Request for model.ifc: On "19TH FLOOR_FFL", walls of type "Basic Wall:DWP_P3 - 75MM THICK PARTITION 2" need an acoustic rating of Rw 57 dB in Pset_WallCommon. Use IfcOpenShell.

First a look at what the model holds.

```python
import ifcopenshell
import ifcopenshell.util.element

model = ifcopenshell.open("model.ifc")
print(model.schema)
storey = next(s for s in model.by_type("IfcBuildingStorey") if s.Name == "19TH FLOOR_FFL")
walls = [e for e in ifcopenshell.util.element.get_decomposition(storey) if e.is_a("IfcWall")]
seen = {}
for e in walls:
    element_type = ifcopenshell.util.element.get_type(e)
    key = (element_type.Name if element_type != e and element_type else None, ifcopenshell.util.element.get_pset(e, "Pset_WallCommon", "AcousticRating"))
    seen[key] = seen.get(key, 0) + 1
for (name, value), count in sorted(seen.items(), key=str):
    print(count, "x", name, "|", value)
```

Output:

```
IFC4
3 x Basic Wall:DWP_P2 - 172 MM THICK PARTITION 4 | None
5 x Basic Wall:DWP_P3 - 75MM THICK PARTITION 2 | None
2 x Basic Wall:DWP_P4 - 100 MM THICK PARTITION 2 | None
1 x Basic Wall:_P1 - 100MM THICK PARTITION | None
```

```python
import ifcopenshell
import ifcopenshell.api.pset
import ifcopenshell.util.element

model = ifcopenshell.open("model.ifc")

storey = next(s for s in model.by_type("IfcBuildingStorey") if s.Name == "19TH FLOOR_FFL")
walls = [e for e in ifcopenshell.util.element.get_decomposition(storey) if e.is_a("IfcWall")]

count = 0
for e in walls:
    element_type = ifcopenshell.util.element.get_type(e)
    if element_type in (None, e) or element_type.Name != "Basic Wall:DWP_P3 - 75MM THICK PARTITION 2":
        continue
    # add_pset returns the element's existing set when there is one.
    pset = ifcopenshell.api.pset.add_pset(model, product=e, name="Pset_WallCommon")
    ifcopenshell.api.pset.edit_pset(model, pset=pset, properties={"AcousticRating": "Rw 57 dB"})
    count += 1

print(count, "walls updated")

model.write("model_updated.ifc")
```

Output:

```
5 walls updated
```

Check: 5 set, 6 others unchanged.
